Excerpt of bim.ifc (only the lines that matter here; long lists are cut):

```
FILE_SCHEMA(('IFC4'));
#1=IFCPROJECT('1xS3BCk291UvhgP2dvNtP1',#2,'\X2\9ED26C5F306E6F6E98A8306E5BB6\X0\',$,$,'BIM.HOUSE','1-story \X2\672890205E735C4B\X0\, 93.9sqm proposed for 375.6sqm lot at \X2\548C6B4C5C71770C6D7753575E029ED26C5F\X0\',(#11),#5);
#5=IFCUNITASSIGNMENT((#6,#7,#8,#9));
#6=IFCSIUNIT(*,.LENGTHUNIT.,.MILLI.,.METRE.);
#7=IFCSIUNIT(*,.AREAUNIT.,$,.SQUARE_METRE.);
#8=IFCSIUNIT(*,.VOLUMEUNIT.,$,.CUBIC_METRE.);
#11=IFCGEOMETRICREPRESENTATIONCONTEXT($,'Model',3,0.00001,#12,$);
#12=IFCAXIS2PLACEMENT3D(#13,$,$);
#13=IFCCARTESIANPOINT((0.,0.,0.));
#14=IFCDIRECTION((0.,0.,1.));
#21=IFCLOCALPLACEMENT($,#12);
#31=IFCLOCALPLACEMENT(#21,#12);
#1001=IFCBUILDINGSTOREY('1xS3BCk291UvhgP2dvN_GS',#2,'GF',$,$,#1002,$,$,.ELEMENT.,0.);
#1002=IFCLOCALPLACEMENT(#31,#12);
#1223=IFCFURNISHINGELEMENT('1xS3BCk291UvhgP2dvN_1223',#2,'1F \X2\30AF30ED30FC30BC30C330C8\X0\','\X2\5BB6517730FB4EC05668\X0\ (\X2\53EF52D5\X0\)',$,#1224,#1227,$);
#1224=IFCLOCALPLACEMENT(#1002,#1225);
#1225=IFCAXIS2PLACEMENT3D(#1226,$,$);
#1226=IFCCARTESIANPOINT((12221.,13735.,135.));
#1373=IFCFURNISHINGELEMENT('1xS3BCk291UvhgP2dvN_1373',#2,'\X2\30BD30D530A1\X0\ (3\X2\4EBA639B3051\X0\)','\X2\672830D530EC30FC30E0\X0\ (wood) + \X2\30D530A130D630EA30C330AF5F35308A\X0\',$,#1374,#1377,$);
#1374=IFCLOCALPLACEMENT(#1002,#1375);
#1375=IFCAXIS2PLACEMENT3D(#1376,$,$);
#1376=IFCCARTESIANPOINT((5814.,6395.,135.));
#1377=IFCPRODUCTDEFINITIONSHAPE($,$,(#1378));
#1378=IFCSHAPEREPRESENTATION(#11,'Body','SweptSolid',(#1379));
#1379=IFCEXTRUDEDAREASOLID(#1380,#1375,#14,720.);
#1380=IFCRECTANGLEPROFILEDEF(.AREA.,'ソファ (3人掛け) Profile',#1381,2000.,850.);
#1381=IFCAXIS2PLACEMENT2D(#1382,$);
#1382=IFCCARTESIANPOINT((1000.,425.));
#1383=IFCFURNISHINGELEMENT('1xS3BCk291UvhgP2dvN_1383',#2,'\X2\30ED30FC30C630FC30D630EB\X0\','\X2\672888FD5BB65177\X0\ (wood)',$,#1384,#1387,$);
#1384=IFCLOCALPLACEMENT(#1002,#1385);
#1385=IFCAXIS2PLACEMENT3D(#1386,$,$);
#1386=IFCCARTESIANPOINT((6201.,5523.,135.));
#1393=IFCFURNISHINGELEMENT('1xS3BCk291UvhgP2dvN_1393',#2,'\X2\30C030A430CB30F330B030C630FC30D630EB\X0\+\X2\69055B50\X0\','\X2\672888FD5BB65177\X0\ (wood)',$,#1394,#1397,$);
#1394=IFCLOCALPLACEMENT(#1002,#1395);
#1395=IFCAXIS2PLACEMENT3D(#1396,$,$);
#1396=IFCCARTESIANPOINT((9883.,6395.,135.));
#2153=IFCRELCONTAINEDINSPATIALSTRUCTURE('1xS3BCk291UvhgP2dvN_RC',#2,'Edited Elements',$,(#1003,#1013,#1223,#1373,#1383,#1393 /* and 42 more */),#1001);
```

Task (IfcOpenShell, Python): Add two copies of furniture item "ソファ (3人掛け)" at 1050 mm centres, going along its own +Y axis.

```python
import ifcopenshell
import ifcopenshell.api.geometry
import ifcopenshell.api.root
import ifcopenshell.util.element
import ifcopenshell.util.placement
import ifcopenshell.util.unit

model = ifcopenshell.open("bim.ifc")
unit_scale = ifcopenshell.util.unit.calculate_unit_scale(model)


def reuse_history(source, copy):
    """copy_class also copies each property set's owner history, people and application; keep the originals."""
    for rel in copy.IsDefinedBy:
        if rel.is_a("IfcRelDefinesByProperties") and (history := rel.RelatingPropertyDefinition.OwnerHistory):
            rel.RelatingPropertyDefinition.OwnerHistory = source.OwnerHistory
            ifcopenshell.util.element.remove_deep2(model, history)


source = model.by_guid("1xS3BCk291UvhgP2dvN_1373")
base = ifcopenshell.util.placement.get_local_placement(source.ObjectPlacement)
step = base[:3, 1] * 1.05 / unit_scale

for i in range(1, 3):
    copy = ifcopenshell.api.root.copy_class(model, product=source)
    copy.Representation = ifcopenshell.util.element.copy_deep(
        model, source.Representation, exclude=["IfcGeometricRepresentationContext", "IfcRepresentationMap"]
    )
    reuse_history(source, copy)
    matrix = base.copy()
    matrix[:3, 3] += i * step
    print("added at", matrix[:3, 3].round(3) + 0.0)
    ifcopenshell.api.geometry.edit_object_placement(model, product=copy, matrix=matrix, is_si=False)

model.write("bim-out.ifc")
```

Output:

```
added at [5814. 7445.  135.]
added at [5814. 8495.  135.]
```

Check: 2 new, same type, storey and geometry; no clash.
